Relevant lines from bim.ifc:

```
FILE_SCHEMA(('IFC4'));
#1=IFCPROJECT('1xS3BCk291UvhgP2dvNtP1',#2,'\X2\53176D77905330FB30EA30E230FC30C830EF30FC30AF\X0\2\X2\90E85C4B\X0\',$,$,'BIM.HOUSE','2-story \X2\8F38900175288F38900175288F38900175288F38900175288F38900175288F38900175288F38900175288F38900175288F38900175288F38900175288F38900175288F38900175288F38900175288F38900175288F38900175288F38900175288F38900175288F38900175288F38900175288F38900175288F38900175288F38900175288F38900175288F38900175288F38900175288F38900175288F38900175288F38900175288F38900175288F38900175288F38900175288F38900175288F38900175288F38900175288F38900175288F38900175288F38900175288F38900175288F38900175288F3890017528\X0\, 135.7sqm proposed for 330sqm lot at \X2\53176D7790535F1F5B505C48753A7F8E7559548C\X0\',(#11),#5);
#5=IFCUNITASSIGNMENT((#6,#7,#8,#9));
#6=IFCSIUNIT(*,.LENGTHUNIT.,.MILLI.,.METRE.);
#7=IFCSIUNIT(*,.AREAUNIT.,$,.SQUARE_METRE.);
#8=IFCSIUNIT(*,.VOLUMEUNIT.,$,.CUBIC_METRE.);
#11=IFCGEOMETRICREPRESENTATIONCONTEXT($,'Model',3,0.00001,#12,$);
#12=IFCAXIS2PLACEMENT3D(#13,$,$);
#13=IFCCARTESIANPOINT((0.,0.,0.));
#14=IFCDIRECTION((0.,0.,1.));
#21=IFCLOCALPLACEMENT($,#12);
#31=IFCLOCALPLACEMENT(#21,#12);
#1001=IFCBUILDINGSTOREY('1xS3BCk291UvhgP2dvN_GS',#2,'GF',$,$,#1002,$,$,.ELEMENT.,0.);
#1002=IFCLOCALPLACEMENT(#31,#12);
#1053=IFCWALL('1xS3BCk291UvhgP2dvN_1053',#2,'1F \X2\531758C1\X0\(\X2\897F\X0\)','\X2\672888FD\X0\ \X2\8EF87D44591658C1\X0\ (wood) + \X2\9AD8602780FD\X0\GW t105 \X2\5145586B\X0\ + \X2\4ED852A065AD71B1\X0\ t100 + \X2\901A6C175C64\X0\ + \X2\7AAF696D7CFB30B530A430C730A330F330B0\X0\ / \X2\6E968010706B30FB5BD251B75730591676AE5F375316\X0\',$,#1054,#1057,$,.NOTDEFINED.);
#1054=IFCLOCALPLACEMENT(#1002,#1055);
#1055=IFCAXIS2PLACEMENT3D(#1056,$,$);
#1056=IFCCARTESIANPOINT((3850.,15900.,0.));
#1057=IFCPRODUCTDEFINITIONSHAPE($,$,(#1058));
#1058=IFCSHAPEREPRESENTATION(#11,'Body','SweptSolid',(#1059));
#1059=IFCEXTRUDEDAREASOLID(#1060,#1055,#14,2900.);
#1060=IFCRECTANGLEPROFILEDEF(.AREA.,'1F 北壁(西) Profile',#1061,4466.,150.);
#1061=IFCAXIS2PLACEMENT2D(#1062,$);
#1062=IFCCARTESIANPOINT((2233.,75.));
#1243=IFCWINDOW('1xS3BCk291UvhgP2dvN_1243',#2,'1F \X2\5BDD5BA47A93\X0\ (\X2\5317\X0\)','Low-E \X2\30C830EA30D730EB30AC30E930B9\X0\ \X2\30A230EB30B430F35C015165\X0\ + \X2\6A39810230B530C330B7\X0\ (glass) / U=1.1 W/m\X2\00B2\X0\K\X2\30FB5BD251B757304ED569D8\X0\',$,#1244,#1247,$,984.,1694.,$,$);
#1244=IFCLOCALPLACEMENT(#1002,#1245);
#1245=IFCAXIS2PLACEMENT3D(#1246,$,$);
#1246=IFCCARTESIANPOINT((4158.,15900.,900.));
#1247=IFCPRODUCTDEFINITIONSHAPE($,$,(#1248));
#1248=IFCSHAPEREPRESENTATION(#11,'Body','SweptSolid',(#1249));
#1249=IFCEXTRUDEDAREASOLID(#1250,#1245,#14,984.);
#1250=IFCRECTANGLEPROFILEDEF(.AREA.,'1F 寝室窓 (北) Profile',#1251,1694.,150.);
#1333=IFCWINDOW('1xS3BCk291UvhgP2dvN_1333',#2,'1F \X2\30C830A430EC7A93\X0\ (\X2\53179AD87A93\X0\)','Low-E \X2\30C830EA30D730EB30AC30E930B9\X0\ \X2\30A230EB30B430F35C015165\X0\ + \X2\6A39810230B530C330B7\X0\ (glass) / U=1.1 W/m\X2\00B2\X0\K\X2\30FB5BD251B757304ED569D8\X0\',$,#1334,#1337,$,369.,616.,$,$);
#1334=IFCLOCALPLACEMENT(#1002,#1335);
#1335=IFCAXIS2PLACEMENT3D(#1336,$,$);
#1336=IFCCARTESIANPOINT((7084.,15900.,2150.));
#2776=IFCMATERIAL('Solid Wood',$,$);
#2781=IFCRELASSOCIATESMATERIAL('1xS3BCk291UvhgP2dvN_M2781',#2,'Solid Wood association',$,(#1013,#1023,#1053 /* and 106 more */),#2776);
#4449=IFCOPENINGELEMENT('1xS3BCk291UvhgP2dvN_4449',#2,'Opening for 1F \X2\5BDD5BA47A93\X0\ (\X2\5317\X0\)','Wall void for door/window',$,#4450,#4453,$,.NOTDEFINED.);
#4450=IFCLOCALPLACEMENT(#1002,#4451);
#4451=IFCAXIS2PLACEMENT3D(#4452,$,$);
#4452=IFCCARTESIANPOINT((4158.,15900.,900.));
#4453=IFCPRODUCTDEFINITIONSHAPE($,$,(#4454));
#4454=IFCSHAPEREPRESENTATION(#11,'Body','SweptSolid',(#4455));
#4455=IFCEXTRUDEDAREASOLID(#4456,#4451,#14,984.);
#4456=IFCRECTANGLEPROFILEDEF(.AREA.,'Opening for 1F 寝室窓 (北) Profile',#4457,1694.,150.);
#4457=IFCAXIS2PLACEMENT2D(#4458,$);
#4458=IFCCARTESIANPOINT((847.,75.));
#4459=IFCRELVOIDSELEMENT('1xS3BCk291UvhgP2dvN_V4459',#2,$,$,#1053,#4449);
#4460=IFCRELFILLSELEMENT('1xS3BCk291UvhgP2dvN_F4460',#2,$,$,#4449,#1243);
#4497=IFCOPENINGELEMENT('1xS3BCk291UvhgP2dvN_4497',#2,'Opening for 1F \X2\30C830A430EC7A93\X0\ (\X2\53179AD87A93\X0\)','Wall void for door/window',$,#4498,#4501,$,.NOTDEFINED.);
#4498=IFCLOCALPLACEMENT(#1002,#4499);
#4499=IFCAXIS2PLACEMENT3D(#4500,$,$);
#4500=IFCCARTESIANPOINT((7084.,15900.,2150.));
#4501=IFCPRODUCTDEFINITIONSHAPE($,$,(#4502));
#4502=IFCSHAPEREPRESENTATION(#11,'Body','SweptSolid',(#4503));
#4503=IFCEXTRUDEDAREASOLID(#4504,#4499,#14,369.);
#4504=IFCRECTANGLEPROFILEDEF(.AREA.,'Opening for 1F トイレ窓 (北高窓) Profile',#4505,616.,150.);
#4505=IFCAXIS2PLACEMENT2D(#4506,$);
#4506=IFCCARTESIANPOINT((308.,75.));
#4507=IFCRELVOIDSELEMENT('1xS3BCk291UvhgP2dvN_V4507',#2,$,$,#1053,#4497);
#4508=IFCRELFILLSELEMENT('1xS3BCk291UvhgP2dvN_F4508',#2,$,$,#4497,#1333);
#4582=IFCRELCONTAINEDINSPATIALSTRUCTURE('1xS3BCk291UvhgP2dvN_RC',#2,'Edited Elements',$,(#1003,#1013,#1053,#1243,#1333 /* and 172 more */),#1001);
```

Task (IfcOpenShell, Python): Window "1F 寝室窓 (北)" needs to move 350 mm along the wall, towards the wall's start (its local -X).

```python
import ifcopenshell
import ifcopenshell.api.geometry
import ifcopenshell.util.placement
import ifcopenshell.util.unit

model = ifcopenshell.open("bim.ifc")
unit_scale = ifcopenshell.util.unit.calculate_unit_scale(model)

window = model.by_guid("1xS3BCk291UvhgP2dvN_1243")
opening = window.FillsVoids[0].RelatingOpeningElement
wall = opening.VoidsElements[0].RelatingBuildingElement

wall_matrix = ifcopenshell.util.placement.get_local_placement(wall.ObjectPlacement)
shift = wall_matrix[:3, 0] * -0.35 / unit_scale
before = ifcopenshell.util.placement.get_local_placement(window.ObjectPlacement)[:3, 3].copy()

# The window is not placed relative to its opening, so move both.
for product in (opening, window):
    matrix = ifcopenshell.util.placement.get_local_placement(product.ObjectPlacement)
    matrix[:3, 3] += shift
    ifcopenshell.api.geometry.edit_object_placement(model, product=product, matrix=matrix, is_si=False)

after = ifcopenshell.util.placement.get_local_placement(window.ObjectPlacement)[:3, 3]
print("window moved by", (after - before).round(3) + 0.0)

model.write("bim_updated.ifc")
```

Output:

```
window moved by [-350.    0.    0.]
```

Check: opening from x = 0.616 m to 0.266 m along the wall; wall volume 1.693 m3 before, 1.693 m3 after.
